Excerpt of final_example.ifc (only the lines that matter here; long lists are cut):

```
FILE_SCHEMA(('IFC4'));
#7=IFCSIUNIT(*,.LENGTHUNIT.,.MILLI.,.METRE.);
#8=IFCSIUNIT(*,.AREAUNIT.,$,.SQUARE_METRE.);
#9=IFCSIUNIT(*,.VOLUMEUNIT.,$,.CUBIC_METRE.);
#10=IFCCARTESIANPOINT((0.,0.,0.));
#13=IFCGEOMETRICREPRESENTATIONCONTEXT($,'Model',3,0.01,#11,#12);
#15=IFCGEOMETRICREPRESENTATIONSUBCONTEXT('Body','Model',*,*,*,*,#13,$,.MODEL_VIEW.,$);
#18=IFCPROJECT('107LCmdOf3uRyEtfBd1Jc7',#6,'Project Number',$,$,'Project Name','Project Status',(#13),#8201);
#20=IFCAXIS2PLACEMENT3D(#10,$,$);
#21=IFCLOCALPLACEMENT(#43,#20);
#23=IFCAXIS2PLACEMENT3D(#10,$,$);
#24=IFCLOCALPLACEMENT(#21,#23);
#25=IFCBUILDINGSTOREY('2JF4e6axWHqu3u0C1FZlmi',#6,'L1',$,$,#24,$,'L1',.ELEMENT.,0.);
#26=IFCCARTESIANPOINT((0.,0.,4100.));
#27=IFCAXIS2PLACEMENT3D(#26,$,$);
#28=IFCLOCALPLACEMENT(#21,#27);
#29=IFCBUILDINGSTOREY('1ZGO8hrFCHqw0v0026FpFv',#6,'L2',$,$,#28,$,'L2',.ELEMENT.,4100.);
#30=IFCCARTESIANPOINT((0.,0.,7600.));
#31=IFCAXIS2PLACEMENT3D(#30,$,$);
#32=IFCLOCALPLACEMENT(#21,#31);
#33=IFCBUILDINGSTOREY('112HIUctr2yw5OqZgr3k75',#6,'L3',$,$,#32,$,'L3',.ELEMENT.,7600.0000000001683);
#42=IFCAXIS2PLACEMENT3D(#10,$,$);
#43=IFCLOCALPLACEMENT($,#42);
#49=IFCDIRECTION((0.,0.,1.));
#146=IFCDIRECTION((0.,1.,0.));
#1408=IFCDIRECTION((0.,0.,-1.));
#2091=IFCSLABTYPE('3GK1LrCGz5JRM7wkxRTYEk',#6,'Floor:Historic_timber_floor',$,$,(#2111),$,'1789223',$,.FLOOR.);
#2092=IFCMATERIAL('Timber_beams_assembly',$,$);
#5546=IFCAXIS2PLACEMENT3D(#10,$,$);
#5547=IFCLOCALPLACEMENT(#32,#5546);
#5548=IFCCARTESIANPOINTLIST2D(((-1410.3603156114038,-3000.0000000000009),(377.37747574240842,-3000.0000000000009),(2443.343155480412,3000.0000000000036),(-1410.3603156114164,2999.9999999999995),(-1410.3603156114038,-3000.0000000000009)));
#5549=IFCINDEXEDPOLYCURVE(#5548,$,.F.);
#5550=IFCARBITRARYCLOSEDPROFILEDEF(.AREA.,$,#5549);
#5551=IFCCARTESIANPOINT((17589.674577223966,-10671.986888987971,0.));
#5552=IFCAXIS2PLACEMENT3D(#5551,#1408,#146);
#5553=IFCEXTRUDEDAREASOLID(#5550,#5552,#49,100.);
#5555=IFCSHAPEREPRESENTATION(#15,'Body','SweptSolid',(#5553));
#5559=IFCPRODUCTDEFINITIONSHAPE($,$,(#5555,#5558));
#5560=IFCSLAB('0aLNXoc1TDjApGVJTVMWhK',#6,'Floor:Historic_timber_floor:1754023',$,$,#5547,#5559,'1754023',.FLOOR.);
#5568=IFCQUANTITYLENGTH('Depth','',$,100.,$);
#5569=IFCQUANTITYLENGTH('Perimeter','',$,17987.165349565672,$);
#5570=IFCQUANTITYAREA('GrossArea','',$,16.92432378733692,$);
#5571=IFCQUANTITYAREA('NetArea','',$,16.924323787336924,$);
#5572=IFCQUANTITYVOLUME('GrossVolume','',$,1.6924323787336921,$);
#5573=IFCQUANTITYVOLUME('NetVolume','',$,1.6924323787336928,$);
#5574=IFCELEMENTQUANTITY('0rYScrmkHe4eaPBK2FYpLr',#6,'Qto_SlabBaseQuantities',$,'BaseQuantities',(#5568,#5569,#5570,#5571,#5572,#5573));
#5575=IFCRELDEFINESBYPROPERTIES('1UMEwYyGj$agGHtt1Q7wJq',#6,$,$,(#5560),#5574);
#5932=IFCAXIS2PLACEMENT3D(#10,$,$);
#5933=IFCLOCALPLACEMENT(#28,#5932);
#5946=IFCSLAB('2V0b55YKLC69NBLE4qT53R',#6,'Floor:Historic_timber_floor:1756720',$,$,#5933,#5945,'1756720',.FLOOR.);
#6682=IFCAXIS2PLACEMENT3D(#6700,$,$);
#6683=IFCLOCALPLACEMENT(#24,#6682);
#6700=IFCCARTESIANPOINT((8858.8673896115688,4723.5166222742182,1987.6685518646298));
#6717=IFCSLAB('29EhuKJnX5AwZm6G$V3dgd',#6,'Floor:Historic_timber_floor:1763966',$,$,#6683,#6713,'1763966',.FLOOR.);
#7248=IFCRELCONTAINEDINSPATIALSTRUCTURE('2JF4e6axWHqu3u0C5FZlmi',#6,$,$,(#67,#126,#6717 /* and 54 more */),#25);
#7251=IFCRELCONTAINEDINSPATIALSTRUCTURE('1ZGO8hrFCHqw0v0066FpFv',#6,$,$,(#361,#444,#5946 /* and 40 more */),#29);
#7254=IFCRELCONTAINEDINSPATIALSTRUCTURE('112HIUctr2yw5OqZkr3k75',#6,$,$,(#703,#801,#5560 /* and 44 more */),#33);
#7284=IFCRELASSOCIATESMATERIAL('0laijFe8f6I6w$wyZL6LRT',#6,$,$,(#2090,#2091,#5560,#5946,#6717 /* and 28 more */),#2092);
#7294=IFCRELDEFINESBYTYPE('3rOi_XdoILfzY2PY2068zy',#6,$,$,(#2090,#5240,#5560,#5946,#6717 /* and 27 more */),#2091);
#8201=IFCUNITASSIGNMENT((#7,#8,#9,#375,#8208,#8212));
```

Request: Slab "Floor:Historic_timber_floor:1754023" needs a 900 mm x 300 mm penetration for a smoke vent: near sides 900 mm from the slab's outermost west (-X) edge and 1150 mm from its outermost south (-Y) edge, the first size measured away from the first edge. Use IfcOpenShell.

```python
import numpy as np
import ifcopenshell
import ifcopenshell.api.feature
import ifcopenshell.api.geometry
import ifcopenshell.api.pset
import ifcopenshell.api.root
import ifcopenshell.geom
import ifcopenshell.util.element
import ifcopenshell.util.placement
import ifcopenshell.util.representation
import ifcopenshell.util.shape
import ifcopenshell.util.unit

model = ifcopenshell.open("final_example.ifc")
unit_scale = ifcopenshell.util.unit.calculate_unit_scale(model)
area_scale = ifcopenshell.util.unit.calculate_unit_scale(model, "AREAUNIT")
volume_scale = ifcopenshell.util.unit.calculate_unit_scale(model, "VOLUMEUNIT")
settings = ifcopenshell.geom.settings()


def volume(element):
    """Net volume in cubic metres, openings subtracted."""
    shape = ifcopenshell.geom.create_shape(settings, element)
    return ifcopenshell.util.shape.get_volume(shape.geometry)


slab = model.by_id(5560)
before = volume(slab)

# Extent in the slab's own axes, in metres. The edges named are its -X and -Y sides.
slab_shape = ifcopenshell.geom.create_shape(settings, slab)
vertices = ifcopenshell.util.shape.get_vertices(slab_shape.geometry)
x_min, y_min, bottom = vertices.min(axis=0)
top = vertices[:, 2].max()

opening = ifcopenshell.api.root.create_entity(model, ifc_class="IfcOpeningElement", name="Smoke vent opening", predefined_type="OPENING")
context = ifcopenshell.util.representation.get_context(model, "Model", "Body", "MODEL_VIEW")
width, depth = 0.9, 0.3
outline = [(0.0, 0.0), (width, 0.0), (width, depth), (0.0, depth), (0.0, 0.0)]
# Overshoot both faces by 50 mm so the cut is clean.
shape = ifcopenshell.api.geometry.add_slab_representation(
    model, context=context, depth=top - bottom + 0.1, polyline=outline
)
ifcopenshell.api.geometry.assign_representation(model, product=opening, representation=shape)

matrix = ifcopenshell.util.placement.get_local_placement(slab.ObjectPlacement)
matrix[:, 3] = matrix @ np.append(np.array([x_min + 0.9, y_min + 1.15, bottom - 0.05]) / unit_scale, 1.0)
ifcopenshell.api.geometry.edit_object_placement(model, product=opening, matrix=matrix, is_si=False)
ifcopenshell.api.feature.add_feature(model, feature=opening, element=slab)

after = volume(slab)

# Update the slab's stored quantities.
qto = model.by_id(ifcopenshell.util.element.get_pset(slab, "Qto_SlabBaseQuantities", should_inherit=False)["id"])
ifcopenshell.api.pset.edit_qto(model, qto=qto, properties={
    "NetArea": after / (top - bottom) / area_scale,
    "NetVolume": after / volume_scale,
})

print(f"slab volume {before:.3f} -> {after:.3f} m3")

model.write("final_example_edited.ifc")
```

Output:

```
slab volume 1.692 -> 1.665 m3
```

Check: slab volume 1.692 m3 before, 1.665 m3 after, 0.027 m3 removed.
